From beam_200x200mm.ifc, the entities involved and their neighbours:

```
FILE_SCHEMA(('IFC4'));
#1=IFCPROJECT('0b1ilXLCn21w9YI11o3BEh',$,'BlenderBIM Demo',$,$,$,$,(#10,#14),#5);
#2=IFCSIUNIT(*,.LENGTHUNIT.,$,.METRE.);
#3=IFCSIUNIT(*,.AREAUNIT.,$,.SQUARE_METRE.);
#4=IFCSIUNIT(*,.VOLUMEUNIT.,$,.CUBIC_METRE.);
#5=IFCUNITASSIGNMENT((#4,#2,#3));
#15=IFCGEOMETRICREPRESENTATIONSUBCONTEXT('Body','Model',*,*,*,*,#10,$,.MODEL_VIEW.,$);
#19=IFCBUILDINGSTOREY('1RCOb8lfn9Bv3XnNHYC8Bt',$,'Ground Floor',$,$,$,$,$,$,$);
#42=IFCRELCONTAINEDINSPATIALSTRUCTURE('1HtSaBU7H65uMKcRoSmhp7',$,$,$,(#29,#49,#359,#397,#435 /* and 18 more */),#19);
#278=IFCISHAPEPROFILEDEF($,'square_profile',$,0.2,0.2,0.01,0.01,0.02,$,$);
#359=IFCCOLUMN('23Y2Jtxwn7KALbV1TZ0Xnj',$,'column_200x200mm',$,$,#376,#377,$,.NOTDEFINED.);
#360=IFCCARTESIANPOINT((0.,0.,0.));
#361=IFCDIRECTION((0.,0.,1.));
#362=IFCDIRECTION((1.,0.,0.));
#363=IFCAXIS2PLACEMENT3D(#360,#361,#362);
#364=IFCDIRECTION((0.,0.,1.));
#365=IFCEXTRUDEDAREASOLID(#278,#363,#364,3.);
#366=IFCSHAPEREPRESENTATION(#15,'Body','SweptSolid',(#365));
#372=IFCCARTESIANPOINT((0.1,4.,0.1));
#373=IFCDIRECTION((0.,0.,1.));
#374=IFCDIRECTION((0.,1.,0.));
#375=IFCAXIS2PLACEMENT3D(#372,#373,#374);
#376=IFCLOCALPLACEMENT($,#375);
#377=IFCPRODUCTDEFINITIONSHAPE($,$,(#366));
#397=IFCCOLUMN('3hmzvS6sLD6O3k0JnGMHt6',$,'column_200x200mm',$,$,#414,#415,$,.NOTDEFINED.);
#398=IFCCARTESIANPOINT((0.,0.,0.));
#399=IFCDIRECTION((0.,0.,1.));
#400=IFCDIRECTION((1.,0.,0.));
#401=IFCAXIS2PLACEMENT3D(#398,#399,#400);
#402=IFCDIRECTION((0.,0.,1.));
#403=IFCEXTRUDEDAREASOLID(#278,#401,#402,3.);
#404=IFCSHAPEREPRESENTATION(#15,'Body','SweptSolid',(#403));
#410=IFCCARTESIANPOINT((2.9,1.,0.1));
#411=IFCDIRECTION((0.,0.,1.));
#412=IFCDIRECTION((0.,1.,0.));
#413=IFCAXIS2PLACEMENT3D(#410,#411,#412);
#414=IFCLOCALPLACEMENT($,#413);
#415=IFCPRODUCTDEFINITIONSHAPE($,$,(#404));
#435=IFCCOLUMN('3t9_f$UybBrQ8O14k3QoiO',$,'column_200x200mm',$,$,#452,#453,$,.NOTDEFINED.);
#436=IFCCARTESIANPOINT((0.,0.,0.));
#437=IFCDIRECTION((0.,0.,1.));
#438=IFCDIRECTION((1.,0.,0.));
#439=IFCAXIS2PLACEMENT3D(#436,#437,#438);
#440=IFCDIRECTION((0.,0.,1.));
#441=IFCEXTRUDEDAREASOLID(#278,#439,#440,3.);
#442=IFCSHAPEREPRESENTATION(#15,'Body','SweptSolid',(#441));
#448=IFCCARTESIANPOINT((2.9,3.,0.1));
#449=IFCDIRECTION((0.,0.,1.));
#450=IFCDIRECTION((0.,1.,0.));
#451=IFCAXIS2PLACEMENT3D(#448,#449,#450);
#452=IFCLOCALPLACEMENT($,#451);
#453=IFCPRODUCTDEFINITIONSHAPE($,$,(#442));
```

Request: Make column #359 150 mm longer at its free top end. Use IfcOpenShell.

```python
import ifcopenshell
import ifcopenshell.util.representation

model = ifcopenshell.open("beam_200x200mm.ifc")

member = model.by_guid("23Y2Jtxwn7KALbV1TZ0Xnj")
change = 0.15

# The extrusion runs towards the end named, so only its depth changes.
body = ifcopenshell.util.representation.get_representation(member, "Model", "Body")
solid = body.Items[0]
old_length = solid.Depth
solid.Depth += change

print(f"length {old_length:g} -> {solid.Depth:g}")

model.write("beam_200x200mm_edited.ifc")
```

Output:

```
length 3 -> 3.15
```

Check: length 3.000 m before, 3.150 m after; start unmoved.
